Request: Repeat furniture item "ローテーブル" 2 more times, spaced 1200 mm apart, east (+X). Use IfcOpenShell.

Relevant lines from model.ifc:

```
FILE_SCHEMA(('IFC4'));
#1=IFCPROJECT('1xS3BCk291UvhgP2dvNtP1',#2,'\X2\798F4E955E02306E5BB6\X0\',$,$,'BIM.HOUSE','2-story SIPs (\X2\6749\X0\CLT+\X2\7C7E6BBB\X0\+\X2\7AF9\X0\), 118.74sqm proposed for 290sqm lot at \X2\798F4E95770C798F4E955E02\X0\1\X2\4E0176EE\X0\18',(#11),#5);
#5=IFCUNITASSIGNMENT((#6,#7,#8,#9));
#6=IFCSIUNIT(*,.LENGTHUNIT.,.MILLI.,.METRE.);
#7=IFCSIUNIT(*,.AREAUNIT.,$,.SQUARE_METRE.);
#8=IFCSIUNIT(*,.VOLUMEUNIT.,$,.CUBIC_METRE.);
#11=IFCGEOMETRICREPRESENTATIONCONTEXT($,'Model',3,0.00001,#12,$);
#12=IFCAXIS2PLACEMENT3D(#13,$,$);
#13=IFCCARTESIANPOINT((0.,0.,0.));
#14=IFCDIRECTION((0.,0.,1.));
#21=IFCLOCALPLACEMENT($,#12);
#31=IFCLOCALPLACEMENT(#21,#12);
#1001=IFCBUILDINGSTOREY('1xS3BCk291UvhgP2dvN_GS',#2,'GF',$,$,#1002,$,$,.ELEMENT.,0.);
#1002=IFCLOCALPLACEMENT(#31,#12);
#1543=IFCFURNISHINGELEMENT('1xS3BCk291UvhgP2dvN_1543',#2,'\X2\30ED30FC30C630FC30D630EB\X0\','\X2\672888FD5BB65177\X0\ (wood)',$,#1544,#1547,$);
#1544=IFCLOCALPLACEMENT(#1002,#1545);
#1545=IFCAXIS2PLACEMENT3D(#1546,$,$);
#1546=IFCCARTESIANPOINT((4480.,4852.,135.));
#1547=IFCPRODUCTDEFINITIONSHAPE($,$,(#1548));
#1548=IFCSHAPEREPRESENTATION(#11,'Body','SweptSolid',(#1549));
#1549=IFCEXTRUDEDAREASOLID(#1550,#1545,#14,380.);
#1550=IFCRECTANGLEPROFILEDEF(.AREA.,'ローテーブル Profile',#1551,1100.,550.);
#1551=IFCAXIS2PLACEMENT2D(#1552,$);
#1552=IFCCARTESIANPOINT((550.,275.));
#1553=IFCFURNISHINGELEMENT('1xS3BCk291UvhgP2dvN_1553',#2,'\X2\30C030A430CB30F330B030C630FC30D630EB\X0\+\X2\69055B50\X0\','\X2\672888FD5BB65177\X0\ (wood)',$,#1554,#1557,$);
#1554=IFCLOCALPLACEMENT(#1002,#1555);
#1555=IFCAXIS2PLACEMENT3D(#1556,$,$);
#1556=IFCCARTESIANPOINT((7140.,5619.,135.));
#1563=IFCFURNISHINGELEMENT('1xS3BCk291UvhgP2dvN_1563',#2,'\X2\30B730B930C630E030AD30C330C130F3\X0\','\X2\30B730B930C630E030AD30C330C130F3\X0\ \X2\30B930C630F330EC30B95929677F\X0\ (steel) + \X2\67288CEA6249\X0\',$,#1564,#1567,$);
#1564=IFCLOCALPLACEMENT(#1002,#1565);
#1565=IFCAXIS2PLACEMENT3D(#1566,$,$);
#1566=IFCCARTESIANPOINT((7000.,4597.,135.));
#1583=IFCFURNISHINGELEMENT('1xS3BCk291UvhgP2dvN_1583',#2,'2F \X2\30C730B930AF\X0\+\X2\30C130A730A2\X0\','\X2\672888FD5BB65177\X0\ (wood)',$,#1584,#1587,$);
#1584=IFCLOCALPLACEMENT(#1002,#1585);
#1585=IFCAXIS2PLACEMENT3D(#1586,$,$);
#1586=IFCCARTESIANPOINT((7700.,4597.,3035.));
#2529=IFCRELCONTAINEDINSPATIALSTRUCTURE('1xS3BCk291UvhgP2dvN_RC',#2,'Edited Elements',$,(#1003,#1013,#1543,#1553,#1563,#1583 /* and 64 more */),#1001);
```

```python
import numpy as np
import ifcopenshell
import ifcopenshell.api.geometry
import ifcopenshell.api.root
import ifcopenshell.util.element
import ifcopenshell.util.placement
import ifcopenshell.util.unit

model = ifcopenshell.open("model.ifc")
unit_scale = ifcopenshell.util.unit.calculate_unit_scale(model)


def reuse_history(source, copy):
    """copy_class also copies each property set's owner history, people and application; keep the originals."""
    for rel in copy.IsDefinedBy:
        if rel.is_a("IfcRelDefinesByProperties") and (history := rel.RelatingPropertyDefinition.OwnerHistory):
            rel.RelatingPropertyDefinition.OwnerHistory = source.OwnerHistory
            ifcopenshell.util.element.remove_deep2(model, history)


source = model.by_guid("1xS3BCk291UvhgP2dvN_1543")
base = ifcopenshell.util.placement.get_local_placement(source.ObjectPlacement)
step = np.array([1.0, 0.0, 0.0]) * 1.2 / unit_scale

for i in range(1, 3):
    copy = ifcopenshell.api.root.copy_class(model, product=source)
    copy.Representation = ifcopenshell.util.element.copy_deep(
        model, source.Representation, exclude=["IfcGeometricRepresentationContext", "IfcRepresentationMap"]
    )
    reuse_history(source, copy)
    matrix = base.copy()
    matrix[:3, 3] += i * step
    print("added at", matrix[:3, 3].round(3) + 0.0)
    ifcopenshell.api.geometry.edit_object_placement(model, product=copy, matrix=matrix, is_si=False)

model.write("model_edited.ifc")
```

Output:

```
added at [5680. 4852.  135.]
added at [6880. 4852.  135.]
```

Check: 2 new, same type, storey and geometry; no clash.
